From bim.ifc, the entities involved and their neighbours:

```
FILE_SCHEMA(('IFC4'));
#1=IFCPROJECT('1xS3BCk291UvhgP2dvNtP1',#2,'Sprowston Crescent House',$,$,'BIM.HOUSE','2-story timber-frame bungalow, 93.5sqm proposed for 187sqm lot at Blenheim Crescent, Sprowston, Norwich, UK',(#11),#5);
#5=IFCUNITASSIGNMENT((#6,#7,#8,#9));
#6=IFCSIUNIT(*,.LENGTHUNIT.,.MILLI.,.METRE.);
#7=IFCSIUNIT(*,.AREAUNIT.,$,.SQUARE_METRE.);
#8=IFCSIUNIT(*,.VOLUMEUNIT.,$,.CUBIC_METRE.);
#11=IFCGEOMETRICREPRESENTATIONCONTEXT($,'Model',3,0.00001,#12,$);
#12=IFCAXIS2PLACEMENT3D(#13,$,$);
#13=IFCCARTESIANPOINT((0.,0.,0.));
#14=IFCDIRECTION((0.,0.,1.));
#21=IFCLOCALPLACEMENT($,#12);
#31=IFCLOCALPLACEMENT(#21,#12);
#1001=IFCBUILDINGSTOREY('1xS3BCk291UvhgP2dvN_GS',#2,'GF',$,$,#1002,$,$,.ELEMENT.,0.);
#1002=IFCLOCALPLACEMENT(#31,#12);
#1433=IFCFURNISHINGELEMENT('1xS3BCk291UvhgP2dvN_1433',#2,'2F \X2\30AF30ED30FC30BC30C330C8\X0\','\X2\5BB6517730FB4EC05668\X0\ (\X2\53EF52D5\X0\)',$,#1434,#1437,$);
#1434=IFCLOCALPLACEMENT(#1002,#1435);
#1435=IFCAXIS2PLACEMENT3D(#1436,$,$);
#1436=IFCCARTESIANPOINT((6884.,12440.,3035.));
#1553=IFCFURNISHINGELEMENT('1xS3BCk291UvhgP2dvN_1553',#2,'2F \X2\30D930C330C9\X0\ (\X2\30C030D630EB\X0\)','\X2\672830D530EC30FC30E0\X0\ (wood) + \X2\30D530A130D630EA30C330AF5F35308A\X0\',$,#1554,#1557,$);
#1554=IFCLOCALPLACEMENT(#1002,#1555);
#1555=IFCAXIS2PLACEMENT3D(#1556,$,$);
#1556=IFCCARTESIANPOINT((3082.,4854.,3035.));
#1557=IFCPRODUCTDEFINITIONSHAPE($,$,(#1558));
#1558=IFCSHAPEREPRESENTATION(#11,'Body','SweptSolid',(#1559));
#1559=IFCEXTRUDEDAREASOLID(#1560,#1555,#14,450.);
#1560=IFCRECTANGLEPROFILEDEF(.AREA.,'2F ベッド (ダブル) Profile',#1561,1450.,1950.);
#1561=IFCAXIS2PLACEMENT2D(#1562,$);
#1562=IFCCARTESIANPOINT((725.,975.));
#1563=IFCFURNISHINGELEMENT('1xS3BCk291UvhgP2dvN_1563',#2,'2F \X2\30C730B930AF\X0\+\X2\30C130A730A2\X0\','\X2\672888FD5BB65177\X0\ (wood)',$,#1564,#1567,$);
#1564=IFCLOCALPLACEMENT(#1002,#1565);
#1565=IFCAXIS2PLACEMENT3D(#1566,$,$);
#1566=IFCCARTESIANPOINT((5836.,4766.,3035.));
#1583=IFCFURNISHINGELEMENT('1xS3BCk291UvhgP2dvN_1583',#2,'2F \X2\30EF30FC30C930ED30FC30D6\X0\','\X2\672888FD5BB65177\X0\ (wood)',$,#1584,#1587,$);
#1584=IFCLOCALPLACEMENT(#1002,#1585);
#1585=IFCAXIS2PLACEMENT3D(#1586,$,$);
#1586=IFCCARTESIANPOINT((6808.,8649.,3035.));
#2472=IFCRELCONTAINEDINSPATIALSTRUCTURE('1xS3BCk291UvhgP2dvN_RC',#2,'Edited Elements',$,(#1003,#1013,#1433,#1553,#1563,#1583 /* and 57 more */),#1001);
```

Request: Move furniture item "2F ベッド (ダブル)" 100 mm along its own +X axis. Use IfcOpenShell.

```python
import ifcopenshell
import ifcopenshell.api.geometry
import ifcopenshell.util.placement
import ifcopenshell.util.unit

model = ifcopenshell.open("bim.ifc")
unit_scale = ifcopenshell.util.unit.calculate_unit_scale(model)

item = model.by_guid("1xS3BCk291UvhgP2dvN_1553")
matrix = ifcopenshell.util.placement.get_local_placement(item.ObjectPlacement)
matrix[:3, 3] += matrix[:3, 0] * 0.1 / unit_scale
ifcopenshell.api.geometry.edit_object_placement(model, product=item, matrix=matrix, is_si=False)

print(ifcopenshell.util.placement.get_local_placement(item.ObjectPlacement).round(3) + 0.0)

model.write("bim-out.ifc")
```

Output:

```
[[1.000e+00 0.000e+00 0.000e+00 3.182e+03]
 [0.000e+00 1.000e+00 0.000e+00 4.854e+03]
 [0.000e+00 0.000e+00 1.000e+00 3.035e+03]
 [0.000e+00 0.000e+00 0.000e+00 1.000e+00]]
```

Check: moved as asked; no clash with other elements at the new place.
